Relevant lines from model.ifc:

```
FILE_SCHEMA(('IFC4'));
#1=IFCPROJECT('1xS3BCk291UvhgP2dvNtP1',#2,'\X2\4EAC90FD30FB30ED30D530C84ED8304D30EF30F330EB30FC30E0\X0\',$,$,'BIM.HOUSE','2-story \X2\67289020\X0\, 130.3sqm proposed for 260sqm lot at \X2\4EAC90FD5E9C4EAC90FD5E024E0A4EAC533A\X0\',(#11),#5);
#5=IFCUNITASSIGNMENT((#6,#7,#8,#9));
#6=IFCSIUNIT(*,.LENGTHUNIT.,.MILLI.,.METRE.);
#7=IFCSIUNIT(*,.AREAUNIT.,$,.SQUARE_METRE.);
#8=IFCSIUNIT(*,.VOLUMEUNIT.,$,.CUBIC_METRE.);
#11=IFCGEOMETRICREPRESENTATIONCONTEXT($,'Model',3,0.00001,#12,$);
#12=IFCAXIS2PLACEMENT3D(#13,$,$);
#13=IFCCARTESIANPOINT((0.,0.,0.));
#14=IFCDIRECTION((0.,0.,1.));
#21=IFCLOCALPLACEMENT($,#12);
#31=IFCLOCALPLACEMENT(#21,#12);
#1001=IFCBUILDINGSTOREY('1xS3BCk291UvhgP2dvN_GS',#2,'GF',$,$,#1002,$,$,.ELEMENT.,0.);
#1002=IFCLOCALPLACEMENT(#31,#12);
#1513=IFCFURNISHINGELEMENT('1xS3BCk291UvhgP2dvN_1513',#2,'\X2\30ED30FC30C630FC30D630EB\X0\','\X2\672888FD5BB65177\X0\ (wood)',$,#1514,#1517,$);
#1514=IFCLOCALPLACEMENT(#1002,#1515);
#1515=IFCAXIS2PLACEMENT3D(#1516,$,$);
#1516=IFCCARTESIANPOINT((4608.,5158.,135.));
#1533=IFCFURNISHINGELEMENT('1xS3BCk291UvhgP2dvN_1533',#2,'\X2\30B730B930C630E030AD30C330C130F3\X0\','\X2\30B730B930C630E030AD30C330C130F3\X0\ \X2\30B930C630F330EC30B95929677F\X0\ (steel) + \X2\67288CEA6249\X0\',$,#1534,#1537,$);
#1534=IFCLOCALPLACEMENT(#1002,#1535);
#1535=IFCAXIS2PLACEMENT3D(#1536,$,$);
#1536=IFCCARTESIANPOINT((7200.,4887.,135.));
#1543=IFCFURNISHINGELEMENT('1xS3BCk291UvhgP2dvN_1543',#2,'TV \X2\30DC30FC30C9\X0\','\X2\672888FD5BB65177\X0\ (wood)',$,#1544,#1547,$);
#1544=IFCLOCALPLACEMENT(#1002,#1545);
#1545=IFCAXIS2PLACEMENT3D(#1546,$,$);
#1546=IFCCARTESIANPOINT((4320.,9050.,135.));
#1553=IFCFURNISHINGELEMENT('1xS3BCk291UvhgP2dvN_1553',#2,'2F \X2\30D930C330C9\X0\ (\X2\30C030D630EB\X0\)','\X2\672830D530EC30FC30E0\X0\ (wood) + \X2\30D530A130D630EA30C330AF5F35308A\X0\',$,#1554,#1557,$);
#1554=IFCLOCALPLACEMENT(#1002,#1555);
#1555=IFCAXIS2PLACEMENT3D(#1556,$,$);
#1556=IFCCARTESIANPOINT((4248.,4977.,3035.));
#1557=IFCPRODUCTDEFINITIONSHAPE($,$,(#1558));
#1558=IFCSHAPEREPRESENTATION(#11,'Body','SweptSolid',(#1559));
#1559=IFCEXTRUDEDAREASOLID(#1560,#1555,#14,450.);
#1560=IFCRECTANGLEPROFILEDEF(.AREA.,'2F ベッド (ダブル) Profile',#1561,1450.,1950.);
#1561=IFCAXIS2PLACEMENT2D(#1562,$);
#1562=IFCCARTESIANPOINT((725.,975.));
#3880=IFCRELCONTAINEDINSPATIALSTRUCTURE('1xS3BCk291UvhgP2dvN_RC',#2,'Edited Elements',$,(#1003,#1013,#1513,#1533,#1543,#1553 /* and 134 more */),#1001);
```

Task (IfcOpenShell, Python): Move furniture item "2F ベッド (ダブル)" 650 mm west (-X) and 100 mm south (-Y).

```python
import ifcopenshell
import ifcopenshell.api.geometry
import ifcopenshell.util.placement
import ifcopenshell.util.unit

model = ifcopenshell.open("model.ifc")
unit_scale = ifcopenshell.util.unit.calculate_unit_scale(model)

item = model.by_guid("1xS3BCk291UvhgP2dvN_1553")
matrix = ifcopenshell.util.placement.get_local_placement(item.ObjectPlacement)
matrix[0, 3] -= 0.65 / unit_scale
matrix[1, 3] -= 0.1 / unit_scale
ifcopenshell.api.geometry.edit_object_placement(model, product=item, matrix=matrix, is_si=False)

print(ifcopenshell.util.placement.get_local_placement(item.ObjectPlacement).round(3) + 0.0)

model.write("model_rev.ifc")
```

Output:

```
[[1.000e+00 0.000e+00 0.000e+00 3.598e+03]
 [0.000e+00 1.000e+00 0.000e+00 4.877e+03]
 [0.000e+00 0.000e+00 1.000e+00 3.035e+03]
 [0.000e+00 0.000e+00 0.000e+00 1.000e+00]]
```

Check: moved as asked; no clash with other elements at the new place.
